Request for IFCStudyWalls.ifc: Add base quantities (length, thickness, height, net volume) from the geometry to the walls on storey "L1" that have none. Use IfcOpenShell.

First a look at what the model holds.

```python
import ifcopenshell
import ifcopenshell.util.element
import ifcopenshell.util.unit

model = ifcopenshell.open("IFCStudyWalls.ifc")
print(model.schema)
for unit_type in ("LENGTHUNIT", "AREAUNIT", "VOLUMEUNIT"):
    print(unit_type, ifcopenshell.util.unit.calculate_unit_scale(model, unit_type))
storey = next(s for s in model.by_type("IfcBuildingStorey") if s.Name == "L1")
walls = [e for e in ifcopenshell.util.element.get_decomposition(storey) if e.is_a("IfcWall")]
for e in sorted(walls, key=lambda e: e.id()):
    print(e.id(), e.is_a(), e.Name, list(ifcopenshell.util.element.get_psets(e, qtos_only=True)), sep=" | ")
```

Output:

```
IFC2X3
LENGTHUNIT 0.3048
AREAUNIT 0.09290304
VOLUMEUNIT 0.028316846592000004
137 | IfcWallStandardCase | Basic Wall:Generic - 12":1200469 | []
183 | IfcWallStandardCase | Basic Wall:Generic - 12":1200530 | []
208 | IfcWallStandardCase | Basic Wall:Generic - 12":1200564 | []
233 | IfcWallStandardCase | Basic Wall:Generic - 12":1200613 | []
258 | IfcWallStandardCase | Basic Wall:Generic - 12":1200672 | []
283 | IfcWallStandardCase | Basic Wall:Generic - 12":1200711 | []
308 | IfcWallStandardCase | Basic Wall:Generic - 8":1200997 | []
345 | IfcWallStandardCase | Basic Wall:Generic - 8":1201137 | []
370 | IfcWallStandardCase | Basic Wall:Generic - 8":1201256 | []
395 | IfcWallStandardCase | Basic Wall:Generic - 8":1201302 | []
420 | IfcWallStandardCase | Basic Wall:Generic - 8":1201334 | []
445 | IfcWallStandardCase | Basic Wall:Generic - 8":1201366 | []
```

```python
import ifcopenshell
import ifcopenshell.api.pset
import ifcopenshell.geom
import ifcopenshell.util.element
import ifcopenshell.util.shape
import ifcopenshell.util.unit

model = ifcopenshell.open("IFCStudyWalls.ifc")
unit_scale = ifcopenshell.util.unit.calculate_unit_scale(model)
volume_scale = ifcopenshell.util.unit.calculate_unit_scale(model, "VOLUMEUNIT")
settings = ifcopenshell.geom.settings()

storey = next(s for s in model.by_type("IfcBuildingStorey") if s.Name == "L1")
walls = [e for e in ifcopenshell.util.element.get_decomposition(storey) if e.is_a("IfcWall")]

for e in sorted(walls, key=lambda e: e.id()):
    if ifcopenshell.util.element.get_psets(e, qtos_only=True, should_inherit=False):
        continue
    # Geometry comes back in metres, in the element's own axes.
    shape = ifcopenshell.geom.create_shape(settings, e)
    values = {
        "Length": ifcopenshell.util.shape.get_x(shape.geometry) / unit_scale,
        "Width": ifcopenshell.util.shape.get_y(shape.geometry) / unit_scale,
        "Height": ifcopenshell.util.shape.get_z(shape.geometry) / unit_scale,
        "NetVolume": ifcopenshell.util.shape.get_volume(shape.geometry) / volume_scale,
    }
    qto = ifcopenshell.api.pset.add_qto(model, product=e, name="BaseQuantities")
    ifcopenshell.api.pset.edit_qto(model, qto=qto, properties=values)
    print(e.id(), {k: round(v, 3) for k, v in values.items()})

model.write("IFCStudyWalls_v2.ifc")
```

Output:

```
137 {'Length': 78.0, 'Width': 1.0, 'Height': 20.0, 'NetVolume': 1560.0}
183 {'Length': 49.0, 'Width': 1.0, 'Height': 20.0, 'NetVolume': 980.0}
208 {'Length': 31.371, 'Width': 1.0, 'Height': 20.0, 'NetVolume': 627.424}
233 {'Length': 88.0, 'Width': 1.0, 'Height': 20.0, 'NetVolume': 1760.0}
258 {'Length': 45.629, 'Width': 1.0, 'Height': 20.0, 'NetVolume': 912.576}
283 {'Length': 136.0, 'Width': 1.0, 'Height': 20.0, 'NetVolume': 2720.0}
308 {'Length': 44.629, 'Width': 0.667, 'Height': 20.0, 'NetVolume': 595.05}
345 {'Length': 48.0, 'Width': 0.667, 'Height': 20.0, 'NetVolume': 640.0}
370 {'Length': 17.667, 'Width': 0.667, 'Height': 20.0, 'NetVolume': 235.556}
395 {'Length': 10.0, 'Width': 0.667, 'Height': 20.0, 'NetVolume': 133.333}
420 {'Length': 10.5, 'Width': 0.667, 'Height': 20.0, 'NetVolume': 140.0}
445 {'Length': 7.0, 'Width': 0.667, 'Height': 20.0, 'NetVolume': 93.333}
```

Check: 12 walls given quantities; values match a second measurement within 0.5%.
